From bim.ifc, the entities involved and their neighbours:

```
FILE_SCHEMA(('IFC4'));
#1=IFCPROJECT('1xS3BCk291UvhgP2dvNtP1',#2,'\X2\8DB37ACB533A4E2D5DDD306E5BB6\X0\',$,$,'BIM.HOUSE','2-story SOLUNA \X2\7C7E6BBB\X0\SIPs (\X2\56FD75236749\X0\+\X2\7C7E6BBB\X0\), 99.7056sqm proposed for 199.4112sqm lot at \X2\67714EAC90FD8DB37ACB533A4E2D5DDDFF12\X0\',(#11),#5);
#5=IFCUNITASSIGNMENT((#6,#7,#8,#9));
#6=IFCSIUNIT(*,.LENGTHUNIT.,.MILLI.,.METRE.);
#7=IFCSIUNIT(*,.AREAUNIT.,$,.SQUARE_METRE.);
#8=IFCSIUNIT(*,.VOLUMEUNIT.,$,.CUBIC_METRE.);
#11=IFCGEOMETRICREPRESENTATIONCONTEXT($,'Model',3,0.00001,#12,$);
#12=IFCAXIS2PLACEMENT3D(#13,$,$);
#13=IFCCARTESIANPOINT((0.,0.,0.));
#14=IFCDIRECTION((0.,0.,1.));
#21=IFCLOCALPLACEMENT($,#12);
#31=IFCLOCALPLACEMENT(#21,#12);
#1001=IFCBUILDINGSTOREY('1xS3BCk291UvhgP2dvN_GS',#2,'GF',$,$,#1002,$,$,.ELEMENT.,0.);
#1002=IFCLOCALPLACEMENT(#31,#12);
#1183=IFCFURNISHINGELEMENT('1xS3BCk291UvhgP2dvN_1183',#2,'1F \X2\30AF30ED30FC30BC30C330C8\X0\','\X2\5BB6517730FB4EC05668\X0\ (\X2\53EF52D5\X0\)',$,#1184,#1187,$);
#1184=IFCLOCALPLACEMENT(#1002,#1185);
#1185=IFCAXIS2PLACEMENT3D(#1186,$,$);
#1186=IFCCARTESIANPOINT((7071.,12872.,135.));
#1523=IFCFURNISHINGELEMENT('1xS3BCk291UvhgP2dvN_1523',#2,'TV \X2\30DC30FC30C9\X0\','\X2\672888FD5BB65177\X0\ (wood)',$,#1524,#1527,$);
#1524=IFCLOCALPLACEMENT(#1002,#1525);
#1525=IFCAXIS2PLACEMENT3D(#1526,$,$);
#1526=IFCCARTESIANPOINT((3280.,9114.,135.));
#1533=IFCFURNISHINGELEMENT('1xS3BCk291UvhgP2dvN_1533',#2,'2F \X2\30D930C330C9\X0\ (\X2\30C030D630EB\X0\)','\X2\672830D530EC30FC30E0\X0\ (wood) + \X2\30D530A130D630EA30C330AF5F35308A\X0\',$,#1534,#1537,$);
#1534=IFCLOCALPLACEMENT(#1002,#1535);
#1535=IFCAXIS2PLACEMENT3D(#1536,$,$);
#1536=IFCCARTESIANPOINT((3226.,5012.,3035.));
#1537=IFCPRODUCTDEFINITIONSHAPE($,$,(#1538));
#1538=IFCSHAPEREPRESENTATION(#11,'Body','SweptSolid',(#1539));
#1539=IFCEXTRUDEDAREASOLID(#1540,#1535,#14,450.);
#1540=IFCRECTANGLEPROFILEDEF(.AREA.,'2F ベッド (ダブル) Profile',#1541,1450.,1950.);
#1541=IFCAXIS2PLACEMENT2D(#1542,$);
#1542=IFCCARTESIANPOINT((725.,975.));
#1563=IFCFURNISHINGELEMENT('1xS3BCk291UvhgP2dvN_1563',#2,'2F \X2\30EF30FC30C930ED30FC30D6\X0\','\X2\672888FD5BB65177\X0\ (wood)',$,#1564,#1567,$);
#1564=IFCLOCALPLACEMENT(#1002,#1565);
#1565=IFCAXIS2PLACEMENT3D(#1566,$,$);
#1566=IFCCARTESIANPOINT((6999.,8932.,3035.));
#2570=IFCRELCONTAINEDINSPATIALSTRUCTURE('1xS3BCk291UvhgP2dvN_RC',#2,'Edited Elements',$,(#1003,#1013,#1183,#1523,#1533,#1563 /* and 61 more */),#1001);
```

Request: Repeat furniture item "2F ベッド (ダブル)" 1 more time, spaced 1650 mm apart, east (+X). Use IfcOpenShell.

```python
import numpy as np
import ifcopenshell
import ifcopenshell.api.geometry
import ifcopenshell.api.root
import ifcopenshell.util.element
import ifcopenshell.util.placement
import ifcopenshell.util.unit

model = ifcopenshell.open("bim.ifc")
unit_scale = ifcopenshell.util.unit.calculate_unit_scale(model)


def reuse_history(source, copy):
    """copy_class also copies each property set's owner history, people and application; keep the originals."""
    for rel in copy.IsDefinedBy:
        if rel.is_a("IfcRelDefinesByProperties") and (history := rel.RelatingPropertyDefinition.OwnerHistory):
            rel.RelatingPropertyDefinition.OwnerHistory = source.OwnerHistory
            ifcopenshell.util.element.remove_deep2(model, history)


source = model.by_guid("1xS3BCk291UvhgP2dvN_1533")
base = ifcopenshell.util.placement.get_local_placement(source.ObjectPlacement)
step = np.array([1.0, 0.0, 0.0]) * 1.65 / unit_scale

for i in range(1, 2):
    copy = ifcopenshell.api.root.copy_class(model, product=source)
    copy.Representation = ifcopenshell.util.element.copy_deep(
        model, source.Representation, exclude=["IfcGeometricRepresentationContext", "IfcRepresentationMap"]
    )
    reuse_history(source, copy)
    matrix = base.copy()
    matrix[:3, 3] += i * step
    print("added at", matrix[:3, 3].round(3) + 0.0)
    ifcopenshell.api.geometry.edit_object_placement(model, product=copy, matrix=matrix, is_si=False)

model.write("bim_rev.ifc")
```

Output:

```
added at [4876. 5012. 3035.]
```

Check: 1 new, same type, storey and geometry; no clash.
